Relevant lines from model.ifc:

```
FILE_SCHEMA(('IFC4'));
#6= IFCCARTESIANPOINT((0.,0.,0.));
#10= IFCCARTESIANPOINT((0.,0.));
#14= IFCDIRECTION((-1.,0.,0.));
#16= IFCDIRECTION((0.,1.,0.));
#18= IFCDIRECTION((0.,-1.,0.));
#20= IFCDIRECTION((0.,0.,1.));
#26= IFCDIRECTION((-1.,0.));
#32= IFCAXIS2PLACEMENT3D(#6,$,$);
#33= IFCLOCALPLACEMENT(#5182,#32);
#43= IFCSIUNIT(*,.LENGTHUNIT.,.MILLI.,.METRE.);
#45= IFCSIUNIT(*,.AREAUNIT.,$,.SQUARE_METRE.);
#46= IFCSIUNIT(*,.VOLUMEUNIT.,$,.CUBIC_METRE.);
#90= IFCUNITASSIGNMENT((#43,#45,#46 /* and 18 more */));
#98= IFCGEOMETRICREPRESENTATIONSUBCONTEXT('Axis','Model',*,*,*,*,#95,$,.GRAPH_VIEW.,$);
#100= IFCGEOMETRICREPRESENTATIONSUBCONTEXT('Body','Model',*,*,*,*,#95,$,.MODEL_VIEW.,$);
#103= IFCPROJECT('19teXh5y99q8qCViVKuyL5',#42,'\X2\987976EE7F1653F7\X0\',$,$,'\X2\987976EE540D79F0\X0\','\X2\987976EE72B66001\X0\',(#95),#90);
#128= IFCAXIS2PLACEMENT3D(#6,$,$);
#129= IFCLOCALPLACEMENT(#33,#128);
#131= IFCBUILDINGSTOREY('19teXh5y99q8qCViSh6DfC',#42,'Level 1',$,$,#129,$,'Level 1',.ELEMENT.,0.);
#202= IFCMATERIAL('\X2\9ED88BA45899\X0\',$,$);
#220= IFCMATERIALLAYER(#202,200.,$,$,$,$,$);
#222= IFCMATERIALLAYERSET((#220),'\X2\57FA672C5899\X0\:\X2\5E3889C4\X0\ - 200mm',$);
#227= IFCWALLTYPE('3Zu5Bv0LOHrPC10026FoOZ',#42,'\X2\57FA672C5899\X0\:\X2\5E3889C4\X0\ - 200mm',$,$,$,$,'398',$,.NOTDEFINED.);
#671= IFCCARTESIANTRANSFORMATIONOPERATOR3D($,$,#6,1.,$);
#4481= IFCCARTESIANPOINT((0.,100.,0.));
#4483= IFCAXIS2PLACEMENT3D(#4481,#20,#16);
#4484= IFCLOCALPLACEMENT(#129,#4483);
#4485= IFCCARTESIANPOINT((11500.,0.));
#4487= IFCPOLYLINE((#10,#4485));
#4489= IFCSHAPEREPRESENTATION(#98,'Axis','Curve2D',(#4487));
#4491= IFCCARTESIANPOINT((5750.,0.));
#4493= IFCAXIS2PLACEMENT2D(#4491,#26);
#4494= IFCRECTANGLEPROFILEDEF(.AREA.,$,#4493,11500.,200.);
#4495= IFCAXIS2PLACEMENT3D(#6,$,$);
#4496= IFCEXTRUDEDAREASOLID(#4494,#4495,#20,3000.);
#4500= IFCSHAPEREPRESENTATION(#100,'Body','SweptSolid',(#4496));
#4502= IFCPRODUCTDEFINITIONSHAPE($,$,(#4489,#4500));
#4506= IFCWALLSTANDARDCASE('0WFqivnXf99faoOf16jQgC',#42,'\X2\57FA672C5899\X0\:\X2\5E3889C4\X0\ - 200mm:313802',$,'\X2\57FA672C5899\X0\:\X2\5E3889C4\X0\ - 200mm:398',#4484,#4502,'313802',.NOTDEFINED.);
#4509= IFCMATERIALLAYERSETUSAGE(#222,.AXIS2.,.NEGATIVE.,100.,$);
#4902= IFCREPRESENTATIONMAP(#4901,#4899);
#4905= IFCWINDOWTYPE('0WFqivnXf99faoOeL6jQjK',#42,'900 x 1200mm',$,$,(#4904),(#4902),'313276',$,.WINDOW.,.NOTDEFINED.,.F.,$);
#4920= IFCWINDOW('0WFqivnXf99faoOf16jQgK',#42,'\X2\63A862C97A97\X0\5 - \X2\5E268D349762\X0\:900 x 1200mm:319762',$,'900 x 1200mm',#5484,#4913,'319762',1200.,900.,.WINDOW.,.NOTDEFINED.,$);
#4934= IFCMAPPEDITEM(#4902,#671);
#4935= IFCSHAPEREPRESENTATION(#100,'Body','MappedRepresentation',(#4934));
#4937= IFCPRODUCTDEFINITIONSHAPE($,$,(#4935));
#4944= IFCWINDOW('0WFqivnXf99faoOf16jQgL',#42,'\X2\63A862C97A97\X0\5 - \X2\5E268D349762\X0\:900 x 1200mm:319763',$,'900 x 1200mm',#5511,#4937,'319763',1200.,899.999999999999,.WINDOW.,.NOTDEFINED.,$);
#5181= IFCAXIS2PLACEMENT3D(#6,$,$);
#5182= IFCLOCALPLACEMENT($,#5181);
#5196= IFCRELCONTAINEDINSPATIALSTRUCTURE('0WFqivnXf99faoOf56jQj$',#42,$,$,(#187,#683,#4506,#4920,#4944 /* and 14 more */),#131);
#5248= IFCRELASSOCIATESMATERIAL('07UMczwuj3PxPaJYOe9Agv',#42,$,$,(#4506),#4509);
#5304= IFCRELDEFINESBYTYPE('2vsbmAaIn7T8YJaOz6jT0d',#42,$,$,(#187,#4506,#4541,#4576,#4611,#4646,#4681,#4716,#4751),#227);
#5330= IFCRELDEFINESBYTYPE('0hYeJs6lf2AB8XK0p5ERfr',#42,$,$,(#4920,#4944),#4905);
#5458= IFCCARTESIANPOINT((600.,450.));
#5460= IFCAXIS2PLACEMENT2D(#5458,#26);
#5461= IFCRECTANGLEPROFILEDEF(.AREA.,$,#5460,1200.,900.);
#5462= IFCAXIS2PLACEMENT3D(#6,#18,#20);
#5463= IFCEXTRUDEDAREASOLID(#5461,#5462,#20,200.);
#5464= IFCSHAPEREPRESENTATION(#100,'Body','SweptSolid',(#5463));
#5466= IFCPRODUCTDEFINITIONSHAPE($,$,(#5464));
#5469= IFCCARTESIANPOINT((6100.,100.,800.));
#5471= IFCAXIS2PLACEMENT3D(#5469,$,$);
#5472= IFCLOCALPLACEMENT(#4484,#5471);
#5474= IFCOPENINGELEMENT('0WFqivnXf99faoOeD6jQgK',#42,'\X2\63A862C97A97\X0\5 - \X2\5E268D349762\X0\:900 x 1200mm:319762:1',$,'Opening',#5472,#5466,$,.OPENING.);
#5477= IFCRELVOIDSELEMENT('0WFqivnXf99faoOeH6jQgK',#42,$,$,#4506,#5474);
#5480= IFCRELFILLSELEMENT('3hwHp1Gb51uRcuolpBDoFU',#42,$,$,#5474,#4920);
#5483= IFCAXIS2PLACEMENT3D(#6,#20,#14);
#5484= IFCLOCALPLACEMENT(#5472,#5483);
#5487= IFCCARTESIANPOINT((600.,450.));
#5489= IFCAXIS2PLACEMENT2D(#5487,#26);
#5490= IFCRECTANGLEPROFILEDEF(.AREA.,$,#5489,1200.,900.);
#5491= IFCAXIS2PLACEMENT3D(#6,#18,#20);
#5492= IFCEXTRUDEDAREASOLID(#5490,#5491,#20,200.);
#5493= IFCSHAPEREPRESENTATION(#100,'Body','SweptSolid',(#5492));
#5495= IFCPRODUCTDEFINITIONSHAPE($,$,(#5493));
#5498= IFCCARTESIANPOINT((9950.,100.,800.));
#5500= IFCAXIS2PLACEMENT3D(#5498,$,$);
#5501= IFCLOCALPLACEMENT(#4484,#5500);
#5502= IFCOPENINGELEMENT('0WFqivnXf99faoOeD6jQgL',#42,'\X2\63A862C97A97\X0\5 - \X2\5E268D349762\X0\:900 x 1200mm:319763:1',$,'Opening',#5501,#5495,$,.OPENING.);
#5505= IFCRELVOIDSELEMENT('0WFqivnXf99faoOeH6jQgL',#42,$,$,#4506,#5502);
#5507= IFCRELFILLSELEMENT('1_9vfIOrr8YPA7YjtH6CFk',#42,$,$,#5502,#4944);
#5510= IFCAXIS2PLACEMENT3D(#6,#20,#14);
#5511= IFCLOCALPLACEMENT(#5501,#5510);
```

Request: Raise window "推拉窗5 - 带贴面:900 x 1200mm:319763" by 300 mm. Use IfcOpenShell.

```python
import numpy as np
import ifcopenshell
import ifcopenshell.api.geometry
import ifcopenshell.util.placement
import ifcopenshell.util.unit

model = ifcopenshell.open("model.ifc")
unit_scale = ifcopenshell.util.unit.calculate_unit_scale(model)

window = model.by_guid("0WFqivnXf99faoOf16jQgL")
opening = window.FillsVoids[0].RelatingOpeningElement
dz = 0.3 / unit_scale

shift = np.array([0.0, 0.0, dz])
# The window is placed relative to its opening, so it follows when the opening moves.
matrix = ifcopenshell.util.placement.get_local_placement(opening.ObjectPlacement)
matrix[:3, 3] += shift
ifcopenshell.api.geometry.edit_object_placement(
    model, product=opening, matrix=matrix, is_si=False, should_transform_children=True
)

print(f"moved by {dz * unit_scale:+.3f} m")

model.write("model_rev.ifc")
```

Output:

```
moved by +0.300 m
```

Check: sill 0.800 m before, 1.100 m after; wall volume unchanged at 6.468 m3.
